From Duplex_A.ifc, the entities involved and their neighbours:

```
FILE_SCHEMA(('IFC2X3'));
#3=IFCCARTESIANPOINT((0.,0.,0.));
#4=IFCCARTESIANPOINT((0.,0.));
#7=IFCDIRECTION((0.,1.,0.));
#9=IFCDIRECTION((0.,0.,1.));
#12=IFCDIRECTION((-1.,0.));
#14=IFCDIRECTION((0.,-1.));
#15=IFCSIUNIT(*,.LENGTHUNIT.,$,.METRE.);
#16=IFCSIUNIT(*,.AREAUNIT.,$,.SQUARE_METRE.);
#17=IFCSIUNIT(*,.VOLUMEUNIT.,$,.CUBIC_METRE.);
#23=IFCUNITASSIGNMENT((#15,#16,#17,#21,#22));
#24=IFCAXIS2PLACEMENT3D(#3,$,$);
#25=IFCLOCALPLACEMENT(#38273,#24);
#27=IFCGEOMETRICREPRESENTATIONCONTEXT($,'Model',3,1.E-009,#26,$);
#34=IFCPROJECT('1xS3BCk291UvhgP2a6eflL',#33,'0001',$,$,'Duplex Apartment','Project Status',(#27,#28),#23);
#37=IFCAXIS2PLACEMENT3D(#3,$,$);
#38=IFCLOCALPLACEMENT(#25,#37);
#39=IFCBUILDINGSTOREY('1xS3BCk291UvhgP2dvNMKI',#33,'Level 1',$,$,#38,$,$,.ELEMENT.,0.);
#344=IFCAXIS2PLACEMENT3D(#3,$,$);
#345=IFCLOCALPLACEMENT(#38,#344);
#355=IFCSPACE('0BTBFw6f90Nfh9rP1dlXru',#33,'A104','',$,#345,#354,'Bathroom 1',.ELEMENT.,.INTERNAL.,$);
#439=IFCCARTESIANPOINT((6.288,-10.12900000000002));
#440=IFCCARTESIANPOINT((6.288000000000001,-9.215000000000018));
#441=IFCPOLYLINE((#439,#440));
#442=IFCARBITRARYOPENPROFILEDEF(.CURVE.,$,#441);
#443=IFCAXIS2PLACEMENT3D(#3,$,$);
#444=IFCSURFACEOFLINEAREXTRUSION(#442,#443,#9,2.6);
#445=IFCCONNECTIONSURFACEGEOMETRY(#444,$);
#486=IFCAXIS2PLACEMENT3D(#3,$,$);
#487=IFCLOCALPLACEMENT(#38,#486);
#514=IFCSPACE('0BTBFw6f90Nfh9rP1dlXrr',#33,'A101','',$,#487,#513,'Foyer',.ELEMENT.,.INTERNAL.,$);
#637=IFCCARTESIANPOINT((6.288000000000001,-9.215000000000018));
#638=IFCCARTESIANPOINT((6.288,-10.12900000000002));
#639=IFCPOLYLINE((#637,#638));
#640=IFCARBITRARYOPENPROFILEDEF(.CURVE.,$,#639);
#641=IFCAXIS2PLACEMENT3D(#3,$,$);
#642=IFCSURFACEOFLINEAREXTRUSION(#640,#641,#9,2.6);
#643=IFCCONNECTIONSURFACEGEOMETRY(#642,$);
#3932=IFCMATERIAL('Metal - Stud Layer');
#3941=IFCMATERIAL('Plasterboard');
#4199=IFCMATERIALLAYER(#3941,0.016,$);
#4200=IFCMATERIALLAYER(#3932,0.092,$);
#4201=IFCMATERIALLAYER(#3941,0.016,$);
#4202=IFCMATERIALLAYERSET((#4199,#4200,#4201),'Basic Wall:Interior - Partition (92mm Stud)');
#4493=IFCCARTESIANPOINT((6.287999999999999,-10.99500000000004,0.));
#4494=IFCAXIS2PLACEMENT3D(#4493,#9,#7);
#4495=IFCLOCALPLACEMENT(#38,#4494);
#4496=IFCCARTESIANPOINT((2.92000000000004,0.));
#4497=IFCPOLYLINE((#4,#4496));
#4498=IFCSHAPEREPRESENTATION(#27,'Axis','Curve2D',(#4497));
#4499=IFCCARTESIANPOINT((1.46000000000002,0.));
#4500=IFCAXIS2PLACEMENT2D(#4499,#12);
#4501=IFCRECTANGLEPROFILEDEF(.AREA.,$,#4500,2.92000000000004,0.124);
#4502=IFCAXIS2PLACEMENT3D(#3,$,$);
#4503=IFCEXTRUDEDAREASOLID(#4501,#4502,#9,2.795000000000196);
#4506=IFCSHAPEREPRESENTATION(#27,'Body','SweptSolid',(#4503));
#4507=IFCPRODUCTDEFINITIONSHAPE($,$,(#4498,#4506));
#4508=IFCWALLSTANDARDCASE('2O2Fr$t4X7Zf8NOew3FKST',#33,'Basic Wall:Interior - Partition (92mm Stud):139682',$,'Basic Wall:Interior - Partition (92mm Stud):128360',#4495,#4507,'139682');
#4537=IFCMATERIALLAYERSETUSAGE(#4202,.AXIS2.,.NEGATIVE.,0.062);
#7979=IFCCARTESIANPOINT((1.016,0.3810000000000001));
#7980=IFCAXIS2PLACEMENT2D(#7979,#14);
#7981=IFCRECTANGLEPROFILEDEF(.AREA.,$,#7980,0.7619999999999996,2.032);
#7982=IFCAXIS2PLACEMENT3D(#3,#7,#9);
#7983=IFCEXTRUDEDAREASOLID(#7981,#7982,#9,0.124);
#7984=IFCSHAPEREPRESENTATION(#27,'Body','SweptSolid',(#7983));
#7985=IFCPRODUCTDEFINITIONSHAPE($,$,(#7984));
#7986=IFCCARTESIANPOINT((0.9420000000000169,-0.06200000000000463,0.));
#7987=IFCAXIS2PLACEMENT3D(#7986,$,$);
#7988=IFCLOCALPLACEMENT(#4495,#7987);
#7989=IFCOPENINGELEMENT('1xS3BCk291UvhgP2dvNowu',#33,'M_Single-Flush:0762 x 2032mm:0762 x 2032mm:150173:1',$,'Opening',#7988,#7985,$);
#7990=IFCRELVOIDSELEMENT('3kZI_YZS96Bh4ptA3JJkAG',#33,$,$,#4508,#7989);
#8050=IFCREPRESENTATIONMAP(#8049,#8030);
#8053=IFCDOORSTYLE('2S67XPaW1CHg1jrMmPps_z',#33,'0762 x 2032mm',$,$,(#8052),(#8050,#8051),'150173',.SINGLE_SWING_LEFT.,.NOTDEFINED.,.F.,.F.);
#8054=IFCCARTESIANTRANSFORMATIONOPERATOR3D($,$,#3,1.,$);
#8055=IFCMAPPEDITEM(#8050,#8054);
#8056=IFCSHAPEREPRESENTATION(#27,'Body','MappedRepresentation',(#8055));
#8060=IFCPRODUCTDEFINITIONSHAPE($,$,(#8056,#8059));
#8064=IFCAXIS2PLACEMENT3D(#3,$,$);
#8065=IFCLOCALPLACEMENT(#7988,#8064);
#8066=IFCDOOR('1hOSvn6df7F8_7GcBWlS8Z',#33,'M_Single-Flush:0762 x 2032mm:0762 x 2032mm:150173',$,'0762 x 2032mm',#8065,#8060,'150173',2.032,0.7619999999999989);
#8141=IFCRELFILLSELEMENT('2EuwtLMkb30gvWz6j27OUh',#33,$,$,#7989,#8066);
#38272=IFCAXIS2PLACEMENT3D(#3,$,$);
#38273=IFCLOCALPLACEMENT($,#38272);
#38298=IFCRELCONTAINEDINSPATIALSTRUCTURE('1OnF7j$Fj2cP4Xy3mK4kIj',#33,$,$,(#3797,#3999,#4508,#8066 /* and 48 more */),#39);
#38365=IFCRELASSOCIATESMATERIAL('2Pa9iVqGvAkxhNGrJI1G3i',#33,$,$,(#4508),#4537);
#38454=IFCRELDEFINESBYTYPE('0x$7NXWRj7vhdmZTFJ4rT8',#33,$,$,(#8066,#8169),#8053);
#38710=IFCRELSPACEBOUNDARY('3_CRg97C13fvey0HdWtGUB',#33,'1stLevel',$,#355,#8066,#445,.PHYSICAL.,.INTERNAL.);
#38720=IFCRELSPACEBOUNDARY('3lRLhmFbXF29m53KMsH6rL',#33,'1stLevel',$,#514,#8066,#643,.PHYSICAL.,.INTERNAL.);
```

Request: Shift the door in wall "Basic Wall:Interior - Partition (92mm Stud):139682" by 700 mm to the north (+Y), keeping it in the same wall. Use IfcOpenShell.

```python
import numpy as np
import ifcopenshell
import ifcopenshell.api.geometry
import ifcopenshell.util.placement

model = ifcopenshell.open("Duplex_A.ifc")

door = model.by_guid("1hOSvn6df7F8_7GcBWlS8Z")
opening = door.FillsVoids[0].RelatingOpeningElement
wall = opening.VoidsElements[0].RelatingBuildingElement

wall_matrix = ifcopenshell.util.placement.get_local_placement(wall.ObjectPlacement)
shift = wall_matrix[:3, 0] * 0.7
before = ifcopenshell.util.placement.get_local_placement(door.ObjectPlacement)[:3, 3].copy()

# The door is placed relative to its opening, so it follows when the opening moves.
matrix = ifcopenshell.util.placement.get_local_placement(opening.ObjectPlacement)
matrix[:3, 3] += shift
ifcopenshell.api.geometry.edit_object_placement(
    model, product=opening, matrix=matrix, is_si=False, should_transform_children=True
)

# Space boundary surfaces are stored in each space's coordinates; move them too.
for rel in door.ProvidesBoundaries:
    if not rel.ConnectionGeometry:
        continue
    surface = rel.ConnectionGeometry.SurfaceOnRelatingElement
    space_matrix = ifcopenshell.util.placement.get_local_placement(rel.RelatingSpace.ObjectPlacement)
    point = np.array(surface.Position.Location.Coordinates) + space_matrix[:3, :3].T @ shift
    surface.Position = model.createIfcAxis2Placement3D(
        model.createIfcCartesianPoint(point.tolist()), surface.Position.Axis, surface.Position.RefDirection
    )

after = ifcopenshell.util.placement.get_local_placement(door.ObjectPlacement)[:3, 3]
print("door moved by", (after - before).round(3) + 0.0)

model.write("Duplex_A_updated.ifc")
```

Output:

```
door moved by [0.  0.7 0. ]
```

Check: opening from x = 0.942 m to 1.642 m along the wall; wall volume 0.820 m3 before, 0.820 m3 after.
